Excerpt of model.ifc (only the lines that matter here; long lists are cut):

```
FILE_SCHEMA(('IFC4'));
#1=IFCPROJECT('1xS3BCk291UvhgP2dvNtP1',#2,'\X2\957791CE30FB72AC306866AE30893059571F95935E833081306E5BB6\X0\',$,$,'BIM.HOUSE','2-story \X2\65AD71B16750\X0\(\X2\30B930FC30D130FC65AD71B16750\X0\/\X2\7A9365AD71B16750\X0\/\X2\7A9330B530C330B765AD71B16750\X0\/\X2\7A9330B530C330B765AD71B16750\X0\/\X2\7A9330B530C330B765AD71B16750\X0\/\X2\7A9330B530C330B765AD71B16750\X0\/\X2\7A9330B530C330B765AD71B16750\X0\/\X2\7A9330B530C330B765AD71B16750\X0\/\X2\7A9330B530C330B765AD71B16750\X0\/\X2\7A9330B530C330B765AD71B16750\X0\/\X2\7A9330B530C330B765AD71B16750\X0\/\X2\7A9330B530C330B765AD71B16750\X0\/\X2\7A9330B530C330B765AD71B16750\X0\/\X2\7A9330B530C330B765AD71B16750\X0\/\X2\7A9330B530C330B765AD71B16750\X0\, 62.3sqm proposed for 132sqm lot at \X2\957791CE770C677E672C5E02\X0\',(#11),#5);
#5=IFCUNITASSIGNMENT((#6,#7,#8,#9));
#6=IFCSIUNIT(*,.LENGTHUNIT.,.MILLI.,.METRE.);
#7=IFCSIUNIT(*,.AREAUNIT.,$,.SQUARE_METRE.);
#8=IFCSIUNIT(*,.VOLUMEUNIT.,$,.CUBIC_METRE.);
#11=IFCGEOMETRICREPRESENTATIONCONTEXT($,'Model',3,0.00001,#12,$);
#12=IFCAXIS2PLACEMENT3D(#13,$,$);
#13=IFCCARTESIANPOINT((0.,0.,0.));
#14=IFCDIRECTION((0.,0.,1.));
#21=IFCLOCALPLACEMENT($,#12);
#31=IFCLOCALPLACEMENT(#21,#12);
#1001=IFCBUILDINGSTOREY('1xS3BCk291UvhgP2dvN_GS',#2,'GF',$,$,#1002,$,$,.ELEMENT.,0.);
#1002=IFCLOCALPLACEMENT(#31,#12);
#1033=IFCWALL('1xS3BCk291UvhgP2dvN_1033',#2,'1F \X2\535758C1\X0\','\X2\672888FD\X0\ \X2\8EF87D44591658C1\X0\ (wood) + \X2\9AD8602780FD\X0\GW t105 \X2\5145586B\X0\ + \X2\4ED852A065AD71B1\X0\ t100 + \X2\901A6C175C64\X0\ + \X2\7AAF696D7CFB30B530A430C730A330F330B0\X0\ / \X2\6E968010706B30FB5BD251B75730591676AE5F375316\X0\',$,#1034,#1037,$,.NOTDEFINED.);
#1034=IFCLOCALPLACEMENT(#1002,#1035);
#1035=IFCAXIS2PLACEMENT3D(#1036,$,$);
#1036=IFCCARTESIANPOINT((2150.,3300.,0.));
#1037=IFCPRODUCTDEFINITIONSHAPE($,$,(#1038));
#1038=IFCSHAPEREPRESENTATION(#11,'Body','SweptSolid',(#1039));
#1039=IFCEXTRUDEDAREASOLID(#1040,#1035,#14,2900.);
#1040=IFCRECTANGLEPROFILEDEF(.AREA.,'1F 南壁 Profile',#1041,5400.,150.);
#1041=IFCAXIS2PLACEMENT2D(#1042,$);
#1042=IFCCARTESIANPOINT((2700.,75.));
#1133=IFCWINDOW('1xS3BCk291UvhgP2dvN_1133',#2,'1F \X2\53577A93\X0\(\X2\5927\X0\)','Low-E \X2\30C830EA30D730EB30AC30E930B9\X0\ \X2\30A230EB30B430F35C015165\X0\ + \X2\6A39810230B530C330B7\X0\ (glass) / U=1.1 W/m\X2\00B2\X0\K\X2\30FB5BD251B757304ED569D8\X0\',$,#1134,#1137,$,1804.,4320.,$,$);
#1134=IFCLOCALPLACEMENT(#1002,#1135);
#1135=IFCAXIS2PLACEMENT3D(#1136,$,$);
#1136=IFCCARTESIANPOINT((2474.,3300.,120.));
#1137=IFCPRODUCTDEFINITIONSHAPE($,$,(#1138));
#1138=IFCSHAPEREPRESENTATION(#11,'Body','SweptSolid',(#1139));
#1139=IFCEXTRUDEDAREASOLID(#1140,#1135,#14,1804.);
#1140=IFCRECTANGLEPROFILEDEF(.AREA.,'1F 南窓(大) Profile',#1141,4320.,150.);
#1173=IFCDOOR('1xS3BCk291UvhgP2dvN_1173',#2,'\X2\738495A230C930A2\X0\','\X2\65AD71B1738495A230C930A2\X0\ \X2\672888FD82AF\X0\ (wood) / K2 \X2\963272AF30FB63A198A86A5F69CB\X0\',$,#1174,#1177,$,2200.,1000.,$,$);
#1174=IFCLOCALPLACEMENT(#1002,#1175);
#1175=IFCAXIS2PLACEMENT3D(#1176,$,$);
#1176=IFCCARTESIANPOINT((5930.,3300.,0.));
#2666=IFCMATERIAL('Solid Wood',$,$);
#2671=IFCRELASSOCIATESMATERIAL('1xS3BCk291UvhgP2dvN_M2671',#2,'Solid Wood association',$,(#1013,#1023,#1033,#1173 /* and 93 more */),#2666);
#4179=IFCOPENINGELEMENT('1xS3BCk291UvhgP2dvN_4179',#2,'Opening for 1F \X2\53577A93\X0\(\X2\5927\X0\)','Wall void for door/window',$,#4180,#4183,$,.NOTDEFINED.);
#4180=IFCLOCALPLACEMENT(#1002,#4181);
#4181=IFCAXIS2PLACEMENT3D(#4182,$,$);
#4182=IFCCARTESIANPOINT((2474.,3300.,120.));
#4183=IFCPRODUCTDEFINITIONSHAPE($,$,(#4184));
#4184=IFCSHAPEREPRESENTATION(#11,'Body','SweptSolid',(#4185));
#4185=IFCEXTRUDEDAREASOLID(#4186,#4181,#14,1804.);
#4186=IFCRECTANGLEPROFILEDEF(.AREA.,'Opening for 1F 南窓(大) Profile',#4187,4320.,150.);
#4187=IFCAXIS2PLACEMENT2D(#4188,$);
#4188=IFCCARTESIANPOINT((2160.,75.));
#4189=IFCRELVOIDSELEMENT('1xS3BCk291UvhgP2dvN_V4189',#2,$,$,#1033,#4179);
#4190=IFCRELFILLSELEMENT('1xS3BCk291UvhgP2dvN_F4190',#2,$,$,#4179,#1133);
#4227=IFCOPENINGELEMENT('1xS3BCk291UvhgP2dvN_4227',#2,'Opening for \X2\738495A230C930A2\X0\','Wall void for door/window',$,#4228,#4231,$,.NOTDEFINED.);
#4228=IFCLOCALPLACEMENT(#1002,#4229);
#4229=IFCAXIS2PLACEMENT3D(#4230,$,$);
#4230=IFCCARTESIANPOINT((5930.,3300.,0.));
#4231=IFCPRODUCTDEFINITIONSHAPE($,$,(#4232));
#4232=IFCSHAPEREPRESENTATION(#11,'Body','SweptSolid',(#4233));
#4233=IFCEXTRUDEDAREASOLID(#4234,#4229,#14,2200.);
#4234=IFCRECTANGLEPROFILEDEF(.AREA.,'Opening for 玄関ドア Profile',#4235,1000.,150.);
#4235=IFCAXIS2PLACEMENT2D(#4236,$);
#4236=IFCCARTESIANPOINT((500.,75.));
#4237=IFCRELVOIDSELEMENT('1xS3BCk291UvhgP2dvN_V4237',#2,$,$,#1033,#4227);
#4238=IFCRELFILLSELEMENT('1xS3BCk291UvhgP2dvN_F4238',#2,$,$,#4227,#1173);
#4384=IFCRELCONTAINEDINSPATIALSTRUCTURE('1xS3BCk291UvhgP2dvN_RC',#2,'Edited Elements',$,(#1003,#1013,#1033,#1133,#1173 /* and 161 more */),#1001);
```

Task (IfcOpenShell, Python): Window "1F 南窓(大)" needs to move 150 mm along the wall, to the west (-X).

```python
import ifcopenshell
import ifcopenshell.api.geometry
import ifcopenshell.util.placement
import ifcopenshell.util.unit

model = ifcopenshell.open("model.ifc")
unit_scale = ifcopenshell.util.unit.calculate_unit_scale(model)

window = model.by_id(1133)
opening = window.FillsVoids[0].RelatingOpeningElement
wall = opening.VoidsElements[0].RelatingBuildingElement

wall_matrix = ifcopenshell.util.placement.get_local_placement(wall.ObjectPlacement)
shift = wall_matrix[:3, 0] * -0.15 / unit_scale
before = ifcopenshell.util.placement.get_local_placement(window.ObjectPlacement)[:3, 3].copy()

# The window is not placed relative to its opening, so move both.
for product in (opening, window):
    matrix = ifcopenshell.util.placement.get_local_placement(product.ObjectPlacement)
    matrix[:3, 3] += shift
    ifcopenshell.api.geometry.edit_object_placement(model, product=product, matrix=matrix, is_si=False)

after = ifcopenshell.util.placement.get_local_placement(window.ObjectPlacement)[:3, 3]
print("window moved by", (after - before).round(3) + 0.0)

model.write("model_updated.ifc")
```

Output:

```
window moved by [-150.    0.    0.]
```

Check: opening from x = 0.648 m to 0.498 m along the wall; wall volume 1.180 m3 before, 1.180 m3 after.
